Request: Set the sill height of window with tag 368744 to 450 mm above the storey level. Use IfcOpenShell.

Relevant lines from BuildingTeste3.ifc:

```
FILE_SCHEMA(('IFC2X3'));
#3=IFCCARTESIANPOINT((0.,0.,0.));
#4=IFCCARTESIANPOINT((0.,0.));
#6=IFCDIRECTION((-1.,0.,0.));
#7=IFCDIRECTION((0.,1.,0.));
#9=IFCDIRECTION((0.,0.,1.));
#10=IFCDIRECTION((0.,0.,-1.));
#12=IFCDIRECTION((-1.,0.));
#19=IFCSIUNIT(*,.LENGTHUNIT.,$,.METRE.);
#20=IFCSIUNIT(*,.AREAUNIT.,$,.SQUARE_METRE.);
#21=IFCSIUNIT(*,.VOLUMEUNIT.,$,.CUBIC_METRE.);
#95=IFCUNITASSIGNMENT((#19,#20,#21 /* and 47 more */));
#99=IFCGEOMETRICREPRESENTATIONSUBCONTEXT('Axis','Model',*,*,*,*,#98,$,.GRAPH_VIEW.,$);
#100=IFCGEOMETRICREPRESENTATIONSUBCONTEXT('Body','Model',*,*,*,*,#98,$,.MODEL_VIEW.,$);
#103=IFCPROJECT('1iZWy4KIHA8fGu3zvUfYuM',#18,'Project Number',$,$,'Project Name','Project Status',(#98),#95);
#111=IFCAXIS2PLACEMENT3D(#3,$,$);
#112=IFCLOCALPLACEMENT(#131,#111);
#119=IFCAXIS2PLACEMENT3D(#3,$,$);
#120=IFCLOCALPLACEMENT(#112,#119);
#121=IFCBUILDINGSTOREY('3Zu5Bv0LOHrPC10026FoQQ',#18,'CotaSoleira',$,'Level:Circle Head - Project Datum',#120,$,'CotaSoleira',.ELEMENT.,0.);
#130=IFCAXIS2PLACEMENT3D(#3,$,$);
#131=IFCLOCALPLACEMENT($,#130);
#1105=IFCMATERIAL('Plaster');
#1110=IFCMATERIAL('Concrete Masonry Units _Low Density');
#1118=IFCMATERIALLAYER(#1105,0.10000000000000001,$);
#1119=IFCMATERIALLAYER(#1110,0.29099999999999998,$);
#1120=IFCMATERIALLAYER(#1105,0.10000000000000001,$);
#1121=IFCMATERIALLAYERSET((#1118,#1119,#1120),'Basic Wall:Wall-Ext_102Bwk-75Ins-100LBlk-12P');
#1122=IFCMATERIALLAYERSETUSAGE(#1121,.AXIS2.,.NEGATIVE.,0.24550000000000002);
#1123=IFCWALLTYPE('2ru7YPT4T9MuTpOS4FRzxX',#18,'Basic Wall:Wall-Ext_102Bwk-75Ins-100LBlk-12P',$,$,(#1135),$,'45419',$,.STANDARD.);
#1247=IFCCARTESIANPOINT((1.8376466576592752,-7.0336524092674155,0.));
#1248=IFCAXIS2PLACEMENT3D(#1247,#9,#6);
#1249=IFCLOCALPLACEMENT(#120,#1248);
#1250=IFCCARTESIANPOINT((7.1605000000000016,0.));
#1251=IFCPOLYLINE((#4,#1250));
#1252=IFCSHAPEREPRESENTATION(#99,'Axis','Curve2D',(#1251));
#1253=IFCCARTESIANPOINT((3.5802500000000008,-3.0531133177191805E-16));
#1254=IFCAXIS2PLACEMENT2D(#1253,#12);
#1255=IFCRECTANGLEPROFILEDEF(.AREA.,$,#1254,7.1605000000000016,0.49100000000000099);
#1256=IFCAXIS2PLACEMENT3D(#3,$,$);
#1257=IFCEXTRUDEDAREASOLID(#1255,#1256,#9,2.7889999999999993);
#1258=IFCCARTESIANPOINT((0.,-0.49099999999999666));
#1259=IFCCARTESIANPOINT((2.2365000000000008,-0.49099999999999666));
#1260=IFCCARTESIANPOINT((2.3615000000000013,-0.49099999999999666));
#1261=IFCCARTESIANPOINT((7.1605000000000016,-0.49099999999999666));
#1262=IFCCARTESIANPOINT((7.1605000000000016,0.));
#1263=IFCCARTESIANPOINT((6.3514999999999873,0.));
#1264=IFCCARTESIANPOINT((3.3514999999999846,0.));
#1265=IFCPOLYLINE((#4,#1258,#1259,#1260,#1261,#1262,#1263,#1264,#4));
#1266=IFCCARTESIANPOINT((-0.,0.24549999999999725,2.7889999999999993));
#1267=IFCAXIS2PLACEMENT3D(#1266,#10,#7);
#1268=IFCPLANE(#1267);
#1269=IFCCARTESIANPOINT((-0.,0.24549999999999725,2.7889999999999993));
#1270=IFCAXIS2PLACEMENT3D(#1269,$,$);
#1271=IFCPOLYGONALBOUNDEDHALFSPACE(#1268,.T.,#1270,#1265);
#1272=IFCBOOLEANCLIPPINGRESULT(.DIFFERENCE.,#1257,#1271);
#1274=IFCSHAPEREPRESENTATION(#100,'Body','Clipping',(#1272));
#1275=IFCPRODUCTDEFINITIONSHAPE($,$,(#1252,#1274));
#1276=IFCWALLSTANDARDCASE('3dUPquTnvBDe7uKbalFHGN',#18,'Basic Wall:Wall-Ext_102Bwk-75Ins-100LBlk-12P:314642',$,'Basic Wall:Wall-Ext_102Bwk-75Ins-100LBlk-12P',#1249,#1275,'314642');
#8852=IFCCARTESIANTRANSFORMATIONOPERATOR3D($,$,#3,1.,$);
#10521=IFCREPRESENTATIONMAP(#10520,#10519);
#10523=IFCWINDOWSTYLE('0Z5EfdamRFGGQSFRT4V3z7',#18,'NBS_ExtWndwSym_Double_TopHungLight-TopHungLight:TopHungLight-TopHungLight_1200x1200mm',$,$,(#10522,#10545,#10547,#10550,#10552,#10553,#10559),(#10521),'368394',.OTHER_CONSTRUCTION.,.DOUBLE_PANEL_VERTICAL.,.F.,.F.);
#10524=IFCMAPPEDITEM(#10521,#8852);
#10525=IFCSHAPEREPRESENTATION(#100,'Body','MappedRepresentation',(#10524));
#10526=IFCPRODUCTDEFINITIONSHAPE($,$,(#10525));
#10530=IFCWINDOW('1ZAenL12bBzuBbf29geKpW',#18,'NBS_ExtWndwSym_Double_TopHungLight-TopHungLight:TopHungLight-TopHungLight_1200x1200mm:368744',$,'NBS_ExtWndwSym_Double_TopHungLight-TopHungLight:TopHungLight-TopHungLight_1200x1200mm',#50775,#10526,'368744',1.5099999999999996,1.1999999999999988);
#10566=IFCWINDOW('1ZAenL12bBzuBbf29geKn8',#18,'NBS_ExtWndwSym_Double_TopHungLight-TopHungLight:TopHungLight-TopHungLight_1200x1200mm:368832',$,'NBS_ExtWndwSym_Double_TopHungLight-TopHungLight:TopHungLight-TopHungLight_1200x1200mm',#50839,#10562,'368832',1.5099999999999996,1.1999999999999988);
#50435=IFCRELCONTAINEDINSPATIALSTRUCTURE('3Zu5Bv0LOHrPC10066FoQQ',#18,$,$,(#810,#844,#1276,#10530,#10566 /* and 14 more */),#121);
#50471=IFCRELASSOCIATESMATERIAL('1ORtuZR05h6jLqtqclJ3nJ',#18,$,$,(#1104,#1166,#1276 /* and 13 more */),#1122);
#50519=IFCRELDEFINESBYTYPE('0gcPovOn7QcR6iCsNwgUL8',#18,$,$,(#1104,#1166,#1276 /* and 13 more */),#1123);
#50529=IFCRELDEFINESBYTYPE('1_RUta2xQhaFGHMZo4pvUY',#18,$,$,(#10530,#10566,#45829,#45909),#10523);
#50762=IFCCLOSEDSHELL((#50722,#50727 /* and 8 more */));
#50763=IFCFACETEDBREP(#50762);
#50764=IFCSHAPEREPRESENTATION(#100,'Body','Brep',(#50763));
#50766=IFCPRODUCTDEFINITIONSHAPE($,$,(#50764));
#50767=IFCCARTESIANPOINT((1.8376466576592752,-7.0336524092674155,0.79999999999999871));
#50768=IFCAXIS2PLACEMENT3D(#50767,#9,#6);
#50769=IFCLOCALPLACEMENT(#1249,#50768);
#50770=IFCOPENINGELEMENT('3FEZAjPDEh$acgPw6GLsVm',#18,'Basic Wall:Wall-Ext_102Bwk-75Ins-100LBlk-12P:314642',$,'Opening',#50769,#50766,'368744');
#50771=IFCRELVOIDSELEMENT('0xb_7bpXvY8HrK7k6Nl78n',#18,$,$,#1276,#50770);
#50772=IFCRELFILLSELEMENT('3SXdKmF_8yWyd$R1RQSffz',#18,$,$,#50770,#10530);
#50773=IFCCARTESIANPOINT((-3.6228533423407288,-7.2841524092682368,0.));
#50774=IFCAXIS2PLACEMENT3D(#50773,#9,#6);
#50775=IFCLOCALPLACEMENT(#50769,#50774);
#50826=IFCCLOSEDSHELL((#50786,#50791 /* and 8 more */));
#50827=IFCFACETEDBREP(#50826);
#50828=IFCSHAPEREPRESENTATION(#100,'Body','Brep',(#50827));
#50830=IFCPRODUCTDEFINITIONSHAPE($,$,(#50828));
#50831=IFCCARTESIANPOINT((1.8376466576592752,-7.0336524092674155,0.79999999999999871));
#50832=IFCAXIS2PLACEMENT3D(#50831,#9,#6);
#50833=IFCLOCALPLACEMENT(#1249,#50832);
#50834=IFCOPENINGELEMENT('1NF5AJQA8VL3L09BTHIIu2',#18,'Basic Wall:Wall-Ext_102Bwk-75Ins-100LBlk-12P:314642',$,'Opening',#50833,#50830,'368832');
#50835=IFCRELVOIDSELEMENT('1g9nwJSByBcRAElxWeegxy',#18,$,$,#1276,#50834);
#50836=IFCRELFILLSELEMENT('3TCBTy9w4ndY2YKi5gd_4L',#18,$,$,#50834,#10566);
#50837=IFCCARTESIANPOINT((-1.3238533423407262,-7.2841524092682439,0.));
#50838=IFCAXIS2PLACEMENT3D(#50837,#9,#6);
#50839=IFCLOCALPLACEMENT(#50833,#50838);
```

```python
import numpy as np
import ifcopenshell
import ifcopenshell.api.geometry
import ifcopenshell.geom
import ifcopenshell.util.element
import ifcopenshell.util.placement
import ifcopenshell.util.shape
import ifcopenshell.util.unit

model = ifcopenshell.open("BuildingTeste3.ifc")
unit_scale = ifcopenshell.util.unit.calculate_unit_scale(model)

window = model.by_guid("1ZAenL12bBzuBbf29geKpW")
opening = window.FillsVoids[0].RelatingOpeningElement
storey = ifcopenshell.util.element.get_container(window, ifc_class="IfcBuildingStorey")
level = ifcopenshell.util.placement.get_local_placement(storey.ObjectPlacement)[2, 3]

# The opening's origin need not be at the sill, so measure its lowest point.
shape = ifcopenshell.geom.create_shape(ifcopenshell.geom.settings(), opening)
bottom = ifcopenshell.util.shape.get_shape_bottom_elevation(shape, shape.geometry) / unit_scale
dz = level + 0.45 / unit_scale - bottom

shift = np.array([0.0, 0.0, dz])
# The window is placed relative to its opening, so it follows when the opening moves.
matrix = ifcopenshell.util.placement.get_local_placement(opening.ObjectPlacement)
matrix[:3, 3] += shift
ifcopenshell.api.geometry.edit_object_placement(
    model, product=opening, matrix=matrix, is_si=False, should_transform_children=True
)

print(f"moved by {dz * unit_scale:+.3f} m")

model.write("BuildingTeste3_v2.ifc")
```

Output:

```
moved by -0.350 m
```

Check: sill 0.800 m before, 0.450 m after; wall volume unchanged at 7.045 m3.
